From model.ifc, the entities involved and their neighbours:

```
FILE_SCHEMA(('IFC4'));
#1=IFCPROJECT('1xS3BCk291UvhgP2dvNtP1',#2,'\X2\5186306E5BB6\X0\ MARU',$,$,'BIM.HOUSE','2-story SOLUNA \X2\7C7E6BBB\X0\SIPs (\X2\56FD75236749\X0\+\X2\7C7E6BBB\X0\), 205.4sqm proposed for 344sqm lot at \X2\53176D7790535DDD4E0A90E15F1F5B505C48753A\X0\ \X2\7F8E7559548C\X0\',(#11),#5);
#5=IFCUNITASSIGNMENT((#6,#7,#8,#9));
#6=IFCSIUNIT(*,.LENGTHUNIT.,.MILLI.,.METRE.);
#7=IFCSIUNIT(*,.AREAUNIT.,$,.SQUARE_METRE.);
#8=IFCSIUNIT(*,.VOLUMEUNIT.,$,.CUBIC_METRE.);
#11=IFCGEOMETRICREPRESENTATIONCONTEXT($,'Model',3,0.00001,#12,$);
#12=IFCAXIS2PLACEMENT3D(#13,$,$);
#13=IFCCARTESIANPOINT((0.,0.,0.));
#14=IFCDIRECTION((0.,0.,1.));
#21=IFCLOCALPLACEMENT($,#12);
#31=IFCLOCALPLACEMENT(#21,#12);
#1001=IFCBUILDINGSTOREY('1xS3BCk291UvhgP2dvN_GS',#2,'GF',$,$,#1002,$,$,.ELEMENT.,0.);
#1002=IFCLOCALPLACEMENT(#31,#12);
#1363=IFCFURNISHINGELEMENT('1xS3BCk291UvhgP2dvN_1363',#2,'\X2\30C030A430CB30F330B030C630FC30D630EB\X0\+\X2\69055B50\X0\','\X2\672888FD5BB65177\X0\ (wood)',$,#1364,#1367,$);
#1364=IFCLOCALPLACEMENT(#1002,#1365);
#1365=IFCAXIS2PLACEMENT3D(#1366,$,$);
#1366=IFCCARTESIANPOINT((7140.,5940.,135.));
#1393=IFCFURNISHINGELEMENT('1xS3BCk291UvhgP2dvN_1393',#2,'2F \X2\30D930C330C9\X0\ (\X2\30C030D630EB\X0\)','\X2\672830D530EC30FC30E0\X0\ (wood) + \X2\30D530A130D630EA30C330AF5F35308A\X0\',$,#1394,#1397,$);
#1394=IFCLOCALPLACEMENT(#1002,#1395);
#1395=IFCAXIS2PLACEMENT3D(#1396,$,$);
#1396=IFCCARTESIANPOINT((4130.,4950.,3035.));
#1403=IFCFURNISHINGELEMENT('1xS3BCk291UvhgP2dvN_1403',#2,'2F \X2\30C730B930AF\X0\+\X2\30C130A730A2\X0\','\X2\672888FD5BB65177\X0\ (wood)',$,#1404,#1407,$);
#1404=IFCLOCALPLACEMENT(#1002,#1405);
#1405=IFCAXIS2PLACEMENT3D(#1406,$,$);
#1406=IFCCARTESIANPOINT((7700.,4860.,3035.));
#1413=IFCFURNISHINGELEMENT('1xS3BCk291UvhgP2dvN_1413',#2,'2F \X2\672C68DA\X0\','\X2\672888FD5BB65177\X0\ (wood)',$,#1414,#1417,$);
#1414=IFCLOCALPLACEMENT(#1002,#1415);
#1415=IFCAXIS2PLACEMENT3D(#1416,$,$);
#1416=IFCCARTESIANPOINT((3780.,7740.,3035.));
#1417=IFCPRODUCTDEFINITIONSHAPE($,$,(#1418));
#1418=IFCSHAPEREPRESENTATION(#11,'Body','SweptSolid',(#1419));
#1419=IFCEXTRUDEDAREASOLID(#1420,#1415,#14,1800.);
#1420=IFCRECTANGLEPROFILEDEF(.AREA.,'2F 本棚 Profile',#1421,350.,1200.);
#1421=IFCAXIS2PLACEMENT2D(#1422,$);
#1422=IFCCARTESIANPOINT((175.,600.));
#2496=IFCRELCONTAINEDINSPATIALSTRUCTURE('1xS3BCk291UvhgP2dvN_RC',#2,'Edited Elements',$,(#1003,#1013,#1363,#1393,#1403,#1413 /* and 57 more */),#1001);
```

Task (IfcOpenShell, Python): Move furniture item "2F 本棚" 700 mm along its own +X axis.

```python
import ifcopenshell
import ifcopenshell.api.geometry
import ifcopenshell.util.placement
import ifcopenshell.util.unit

model = ifcopenshell.open("model.ifc")
unit_scale = ifcopenshell.util.unit.calculate_unit_scale(model)

item = model.by_id(1413)
matrix = ifcopenshell.util.placement.get_local_placement(item.ObjectPlacement)
matrix[:3, 3] += matrix[:3, 0] * 0.7 / unit_scale
ifcopenshell.api.geometry.edit_object_placement(model, product=item, matrix=matrix, is_si=False)

print(ifcopenshell.util.placement.get_local_placement(item.ObjectPlacement).round(3) + 0.0)

model.write("model_edited.ifc")
```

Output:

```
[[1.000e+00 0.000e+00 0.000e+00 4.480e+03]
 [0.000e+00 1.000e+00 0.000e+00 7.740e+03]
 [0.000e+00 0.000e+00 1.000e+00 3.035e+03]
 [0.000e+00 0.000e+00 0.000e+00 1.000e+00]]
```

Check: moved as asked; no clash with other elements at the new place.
